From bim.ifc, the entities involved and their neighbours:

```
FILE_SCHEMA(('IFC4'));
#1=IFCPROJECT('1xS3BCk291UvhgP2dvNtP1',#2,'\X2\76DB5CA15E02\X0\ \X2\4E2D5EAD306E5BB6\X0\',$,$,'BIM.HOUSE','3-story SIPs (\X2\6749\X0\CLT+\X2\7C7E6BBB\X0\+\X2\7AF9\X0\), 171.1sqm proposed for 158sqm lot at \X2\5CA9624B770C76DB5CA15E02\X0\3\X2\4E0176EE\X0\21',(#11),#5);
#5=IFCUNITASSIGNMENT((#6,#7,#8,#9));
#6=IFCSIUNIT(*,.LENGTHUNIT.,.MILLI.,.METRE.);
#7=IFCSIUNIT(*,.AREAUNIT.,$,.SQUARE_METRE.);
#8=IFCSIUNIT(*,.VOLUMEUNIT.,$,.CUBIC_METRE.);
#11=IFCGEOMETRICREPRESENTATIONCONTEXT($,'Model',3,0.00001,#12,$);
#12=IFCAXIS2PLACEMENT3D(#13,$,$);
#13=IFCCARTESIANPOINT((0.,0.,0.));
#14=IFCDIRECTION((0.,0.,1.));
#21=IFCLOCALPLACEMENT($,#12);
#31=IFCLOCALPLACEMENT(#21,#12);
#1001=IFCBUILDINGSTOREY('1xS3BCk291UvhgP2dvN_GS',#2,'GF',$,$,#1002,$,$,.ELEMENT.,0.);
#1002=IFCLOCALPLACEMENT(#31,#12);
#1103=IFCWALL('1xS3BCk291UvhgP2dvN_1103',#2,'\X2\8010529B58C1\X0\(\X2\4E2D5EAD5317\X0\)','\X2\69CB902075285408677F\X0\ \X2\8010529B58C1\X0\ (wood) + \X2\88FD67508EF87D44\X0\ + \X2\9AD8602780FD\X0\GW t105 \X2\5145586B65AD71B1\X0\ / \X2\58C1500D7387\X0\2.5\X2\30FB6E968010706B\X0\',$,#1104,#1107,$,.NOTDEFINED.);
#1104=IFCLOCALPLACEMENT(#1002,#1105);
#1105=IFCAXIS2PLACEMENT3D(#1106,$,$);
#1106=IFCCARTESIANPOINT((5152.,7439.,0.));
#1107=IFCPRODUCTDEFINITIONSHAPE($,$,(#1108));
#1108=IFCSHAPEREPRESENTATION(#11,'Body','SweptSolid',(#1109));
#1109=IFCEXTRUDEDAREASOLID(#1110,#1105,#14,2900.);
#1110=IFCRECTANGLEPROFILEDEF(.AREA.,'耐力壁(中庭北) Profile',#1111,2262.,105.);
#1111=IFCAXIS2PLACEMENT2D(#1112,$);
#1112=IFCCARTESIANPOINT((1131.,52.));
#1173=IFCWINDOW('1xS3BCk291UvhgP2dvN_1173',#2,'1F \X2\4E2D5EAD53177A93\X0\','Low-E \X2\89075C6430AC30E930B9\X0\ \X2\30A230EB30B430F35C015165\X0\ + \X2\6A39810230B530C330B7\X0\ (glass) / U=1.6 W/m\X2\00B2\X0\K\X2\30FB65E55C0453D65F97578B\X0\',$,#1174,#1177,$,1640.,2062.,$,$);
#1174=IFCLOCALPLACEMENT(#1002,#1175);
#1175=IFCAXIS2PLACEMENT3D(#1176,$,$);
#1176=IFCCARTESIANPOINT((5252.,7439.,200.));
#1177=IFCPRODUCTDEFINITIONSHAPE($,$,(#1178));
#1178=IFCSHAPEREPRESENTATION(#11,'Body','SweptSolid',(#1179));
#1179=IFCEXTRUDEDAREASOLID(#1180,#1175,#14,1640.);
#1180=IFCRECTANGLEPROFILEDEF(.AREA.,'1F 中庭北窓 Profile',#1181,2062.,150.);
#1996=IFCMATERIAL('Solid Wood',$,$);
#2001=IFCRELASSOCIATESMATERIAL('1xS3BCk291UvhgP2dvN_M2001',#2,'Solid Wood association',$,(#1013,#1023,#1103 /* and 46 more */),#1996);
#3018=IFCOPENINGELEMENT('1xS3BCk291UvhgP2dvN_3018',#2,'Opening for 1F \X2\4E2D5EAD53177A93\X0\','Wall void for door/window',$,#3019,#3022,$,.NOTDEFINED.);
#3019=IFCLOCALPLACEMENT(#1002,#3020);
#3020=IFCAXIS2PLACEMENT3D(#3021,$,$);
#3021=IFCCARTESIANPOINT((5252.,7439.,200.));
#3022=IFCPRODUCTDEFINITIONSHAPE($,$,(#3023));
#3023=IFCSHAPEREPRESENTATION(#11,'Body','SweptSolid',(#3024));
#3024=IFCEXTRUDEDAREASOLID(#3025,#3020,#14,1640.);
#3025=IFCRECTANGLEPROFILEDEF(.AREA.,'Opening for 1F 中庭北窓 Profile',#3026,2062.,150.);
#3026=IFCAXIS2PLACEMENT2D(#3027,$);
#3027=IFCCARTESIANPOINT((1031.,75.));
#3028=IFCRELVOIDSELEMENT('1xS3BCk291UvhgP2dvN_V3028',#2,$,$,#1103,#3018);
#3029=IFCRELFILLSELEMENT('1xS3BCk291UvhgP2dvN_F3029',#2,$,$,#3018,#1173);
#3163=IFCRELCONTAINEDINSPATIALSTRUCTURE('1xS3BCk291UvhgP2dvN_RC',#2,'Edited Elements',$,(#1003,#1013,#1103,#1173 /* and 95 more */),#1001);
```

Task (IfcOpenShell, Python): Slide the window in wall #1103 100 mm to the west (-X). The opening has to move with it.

```python
import ifcopenshell
import ifcopenshell.api.geometry
import ifcopenshell.util.placement

model = ifcopenshell.open("bim.ifc")

window = model.by_guid("1xS3BCk291UvhgP2dvN_1173")
opening = window.FillsVoids[0].RelatingOpeningElement
wall = opening.VoidsElements[0].RelatingBuildingElement

wall_matrix = ifcopenshell.util.placement.get_local_placement(wall.ObjectPlacement)
shift = wall_matrix[:3, 0] * -100.0
before = ifcopenshell.util.placement.get_local_placement(window.ObjectPlacement)[:3, 3].copy()

# The window is not placed relative to its opening, so move both.
for product in (opening, window):
    matrix = ifcopenshell.util.placement.get_local_placement(product.ObjectPlacement)
    matrix[:3, 3] += shift
    ifcopenshell.api.geometry.edit_object_placement(model, product=product, matrix=matrix, is_si=False)

after = ifcopenshell.util.placement.get_local_placement(window.ObjectPlacement)[:3, 3]
print("window moved by", (after - before).round(3) + 0.0)

model.write("bim_updated.ifc")
```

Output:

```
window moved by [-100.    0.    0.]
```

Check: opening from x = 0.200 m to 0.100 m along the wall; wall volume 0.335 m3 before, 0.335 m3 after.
